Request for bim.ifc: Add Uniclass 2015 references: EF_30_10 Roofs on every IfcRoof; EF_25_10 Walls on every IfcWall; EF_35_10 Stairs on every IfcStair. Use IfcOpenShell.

First a look at what the model holds.

```python
import ifcopenshell

model = ifcopenshell.open("bim.ifc")
print(model.schema)
print("classifications:", [c.Name for c in model.by_type("IfcClassification")])
for ifc_class in ("IfcDoor", "IfcRoof", "IfcStair", "IfcWall", "IfcWindow"):
    print(ifc_class, len(model.by_type(ifc_class)))
```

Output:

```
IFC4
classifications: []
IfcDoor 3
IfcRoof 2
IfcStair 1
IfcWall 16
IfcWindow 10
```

```python
import ifcopenshell
import ifcopenshell.api.classification

model = ifcopenshell.open("bim.ifc")

system = ifcopenshell.api.classification.add_classification(model, classification="Uniclass 2015")

codes = {
    "IfcRoof": ("EF_30_10", "Roofs"),
    "IfcWall": ("EF_25_10", "Walls"),
    "IfcStair": ("EF_35_10", "Stairs"),
}
for ifc_class, (code, name) in codes.items():
    products = model.by_type(ifc_class)
    ifcopenshell.api.classification.add_reference(
        model, products=products, classification=system, identification=code, name=name
    )
    print(code, len(products))

model.write("bim-out.ifc")
```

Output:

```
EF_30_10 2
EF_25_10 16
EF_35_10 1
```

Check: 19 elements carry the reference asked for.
